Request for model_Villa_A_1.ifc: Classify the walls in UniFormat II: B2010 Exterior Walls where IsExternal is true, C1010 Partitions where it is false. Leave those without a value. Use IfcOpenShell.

First a look at what the model holds.

```python
import ifcopenshell
import ifcopenshell.util.element

model = ifcopenshell.open("model_Villa_A_1.ifc")
print(model.schema)
print("classifications:", [c.Name for c in model.by_type("IfcClassification")])
values = [ifcopenshell.util.element.get_pset(e, "Pset_WallCommon", "IsExternal") for e in model.by_type("IfcWall")]
for value in (True, False, None):
    print("IsExternal", value, values.count(value))
```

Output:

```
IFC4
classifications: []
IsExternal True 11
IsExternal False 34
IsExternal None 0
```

```python
import ifcopenshell
import ifcopenshell.api.classification
import ifcopenshell.util.element

model = ifcopenshell.open("model_Villa_A_1.ifc")

system = ifcopenshell.api.classification.add_classification(model, classification="UniFormat II")

walls = model.by_type("IfcWall")
external = {e: ifcopenshell.util.element.get_pset(e, "Pset_WallCommon", "IsExternal") for e in walls}
for flag, code, name in ((True, "B2010", "Exterior Walls"), (False, "C1010", "Partitions")):
    products = [e for e in walls if external[e] is flag]
    ifcopenshell.api.classification.add_reference(
        model, products=products, classification=system, identification=code, name=name
    )
    print(code, len(products))

model.write("model_Villa_A_1_updated.ifc")
```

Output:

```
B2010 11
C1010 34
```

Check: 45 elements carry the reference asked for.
